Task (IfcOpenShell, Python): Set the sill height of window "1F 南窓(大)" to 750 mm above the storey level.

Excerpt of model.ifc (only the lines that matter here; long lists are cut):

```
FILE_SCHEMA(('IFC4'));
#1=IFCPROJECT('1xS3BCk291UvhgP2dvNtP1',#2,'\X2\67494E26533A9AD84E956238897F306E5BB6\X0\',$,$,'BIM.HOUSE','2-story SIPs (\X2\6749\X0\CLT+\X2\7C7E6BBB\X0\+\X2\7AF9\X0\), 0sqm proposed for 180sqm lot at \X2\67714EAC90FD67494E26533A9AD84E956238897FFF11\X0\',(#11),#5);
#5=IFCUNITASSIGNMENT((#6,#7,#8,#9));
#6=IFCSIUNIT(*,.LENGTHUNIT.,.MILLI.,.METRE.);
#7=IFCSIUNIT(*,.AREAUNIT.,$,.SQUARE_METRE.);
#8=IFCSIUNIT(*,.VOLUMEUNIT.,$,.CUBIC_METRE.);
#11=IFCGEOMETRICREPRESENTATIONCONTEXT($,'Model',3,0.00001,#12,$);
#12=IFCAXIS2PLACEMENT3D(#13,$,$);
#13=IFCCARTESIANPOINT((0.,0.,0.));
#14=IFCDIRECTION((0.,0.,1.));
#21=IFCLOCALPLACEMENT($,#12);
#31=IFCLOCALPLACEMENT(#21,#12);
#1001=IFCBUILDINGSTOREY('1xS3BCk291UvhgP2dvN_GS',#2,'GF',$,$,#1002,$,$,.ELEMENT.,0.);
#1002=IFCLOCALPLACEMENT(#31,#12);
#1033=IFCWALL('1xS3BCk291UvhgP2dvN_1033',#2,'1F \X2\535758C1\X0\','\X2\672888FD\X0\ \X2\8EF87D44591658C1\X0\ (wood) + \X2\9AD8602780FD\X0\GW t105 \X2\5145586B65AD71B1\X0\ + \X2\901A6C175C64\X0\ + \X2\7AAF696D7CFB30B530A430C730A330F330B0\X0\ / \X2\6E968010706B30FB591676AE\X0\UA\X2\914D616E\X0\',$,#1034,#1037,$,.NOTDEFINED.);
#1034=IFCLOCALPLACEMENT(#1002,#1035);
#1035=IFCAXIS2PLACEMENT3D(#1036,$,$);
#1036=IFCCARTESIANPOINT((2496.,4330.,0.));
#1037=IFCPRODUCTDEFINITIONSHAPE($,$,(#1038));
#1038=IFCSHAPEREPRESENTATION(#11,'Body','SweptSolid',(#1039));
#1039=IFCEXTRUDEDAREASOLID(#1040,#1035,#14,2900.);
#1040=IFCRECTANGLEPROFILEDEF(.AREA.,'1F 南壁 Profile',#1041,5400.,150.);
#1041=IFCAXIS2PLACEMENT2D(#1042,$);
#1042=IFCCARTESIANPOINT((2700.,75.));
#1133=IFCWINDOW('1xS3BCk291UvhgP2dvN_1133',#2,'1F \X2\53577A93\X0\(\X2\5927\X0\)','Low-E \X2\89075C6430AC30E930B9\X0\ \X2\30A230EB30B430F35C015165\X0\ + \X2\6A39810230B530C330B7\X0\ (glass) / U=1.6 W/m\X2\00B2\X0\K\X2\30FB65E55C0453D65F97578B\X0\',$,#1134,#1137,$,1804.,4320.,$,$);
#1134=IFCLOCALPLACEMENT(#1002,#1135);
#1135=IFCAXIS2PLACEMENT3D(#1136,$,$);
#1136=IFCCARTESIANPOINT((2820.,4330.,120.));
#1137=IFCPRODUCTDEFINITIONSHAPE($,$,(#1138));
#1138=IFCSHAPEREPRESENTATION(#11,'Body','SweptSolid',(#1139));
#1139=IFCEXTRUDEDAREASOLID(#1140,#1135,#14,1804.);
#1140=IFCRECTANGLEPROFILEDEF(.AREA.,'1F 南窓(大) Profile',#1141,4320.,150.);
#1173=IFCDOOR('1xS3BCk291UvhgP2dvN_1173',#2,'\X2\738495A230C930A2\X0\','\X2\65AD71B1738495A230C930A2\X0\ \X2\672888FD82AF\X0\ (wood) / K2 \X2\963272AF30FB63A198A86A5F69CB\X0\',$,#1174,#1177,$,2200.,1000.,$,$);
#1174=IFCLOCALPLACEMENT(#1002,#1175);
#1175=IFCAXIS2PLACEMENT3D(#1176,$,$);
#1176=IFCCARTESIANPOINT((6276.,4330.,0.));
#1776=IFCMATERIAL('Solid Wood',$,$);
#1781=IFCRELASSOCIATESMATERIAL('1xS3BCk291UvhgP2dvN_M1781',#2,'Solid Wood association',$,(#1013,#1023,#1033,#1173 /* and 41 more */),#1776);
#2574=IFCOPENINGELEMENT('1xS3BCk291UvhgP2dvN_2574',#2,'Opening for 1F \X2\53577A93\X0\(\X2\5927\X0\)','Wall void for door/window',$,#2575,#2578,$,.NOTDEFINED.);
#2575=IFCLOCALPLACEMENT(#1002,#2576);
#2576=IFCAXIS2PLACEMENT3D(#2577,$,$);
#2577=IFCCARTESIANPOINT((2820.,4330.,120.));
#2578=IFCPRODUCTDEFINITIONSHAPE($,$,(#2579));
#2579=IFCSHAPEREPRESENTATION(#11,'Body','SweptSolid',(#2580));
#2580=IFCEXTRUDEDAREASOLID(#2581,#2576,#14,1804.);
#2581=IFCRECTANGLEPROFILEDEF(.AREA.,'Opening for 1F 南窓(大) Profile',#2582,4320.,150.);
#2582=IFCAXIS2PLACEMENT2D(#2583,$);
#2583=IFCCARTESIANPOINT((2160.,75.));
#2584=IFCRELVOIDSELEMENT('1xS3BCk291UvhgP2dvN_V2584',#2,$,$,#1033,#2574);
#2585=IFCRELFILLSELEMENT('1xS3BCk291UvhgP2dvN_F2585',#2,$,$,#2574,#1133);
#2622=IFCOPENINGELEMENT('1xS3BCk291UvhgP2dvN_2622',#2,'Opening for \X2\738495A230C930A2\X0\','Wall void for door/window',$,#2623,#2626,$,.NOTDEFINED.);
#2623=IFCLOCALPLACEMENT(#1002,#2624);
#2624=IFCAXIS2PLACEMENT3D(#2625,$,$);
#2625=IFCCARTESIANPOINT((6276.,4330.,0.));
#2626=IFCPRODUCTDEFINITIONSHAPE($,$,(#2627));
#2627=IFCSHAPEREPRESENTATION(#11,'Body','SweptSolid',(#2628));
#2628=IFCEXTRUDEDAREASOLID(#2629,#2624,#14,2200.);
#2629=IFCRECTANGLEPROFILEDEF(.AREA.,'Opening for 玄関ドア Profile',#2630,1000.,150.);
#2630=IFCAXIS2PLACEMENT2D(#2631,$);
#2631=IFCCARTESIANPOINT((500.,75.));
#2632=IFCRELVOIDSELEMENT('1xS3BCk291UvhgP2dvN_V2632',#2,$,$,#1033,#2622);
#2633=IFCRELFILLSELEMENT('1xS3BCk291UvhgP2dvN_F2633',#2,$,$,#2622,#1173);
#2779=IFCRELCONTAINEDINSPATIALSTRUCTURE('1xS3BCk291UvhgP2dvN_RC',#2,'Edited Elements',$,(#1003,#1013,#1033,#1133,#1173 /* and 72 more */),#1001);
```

```python
import numpy as np
import ifcopenshell
import ifcopenshell.api.geometry
import ifcopenshell.geom
import ifcopenshell.util.element
import ifcopenshell.util.placement
import ifcopenshell.util.shape
import ifcopenshell.util.unit

model = ifcopenshell.open("model.ifc")
unit_scale = ifcopenshell.util.unit.calculate_unit_scale(model)

window = model.by_guid("1xS3BCk291UvhgP2dvN_1133")
opening = window.FillsVoids[0].RelatingOpeningElement
storey = ifcopenshell.util.element.get_container(window, ifc_class="IfcBuildingStorey")
level = ifcopenshell.util.placement.get_local_placement(storey.ObjectPlacement)[2, 3]

# The opening's origin need not be at the sill, so measure its lowest point.
shape = ifcopenshell.geom.create_shape(ifcopenshell.geom.settings(), opening)
bottom = ifcopenshell.util.shape.get_shape_bottom_elevation(shape, shape.geometry) / unit_scale
dz = level + 0.75 / unit_scale - bottom

shift = np.array([0.0, 0.0, dz])
# The window is not placed relative to its opening, so move both.
for product in (opening, window):
    matrix = ifcopenshell.util.placement.get_local_placement(product.ObjectPlacement)
    matrix[:3, 3] += shift
    ifcopenshell.api.geometry.edit_object_placement(model, product=product, matrix=matrix, is_si=False)

print(f"moved by {dz * unit_scale:+.3f} m")

model.write("model_rev.ifc")
```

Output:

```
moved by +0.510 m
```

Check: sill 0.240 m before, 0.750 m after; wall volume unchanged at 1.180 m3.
